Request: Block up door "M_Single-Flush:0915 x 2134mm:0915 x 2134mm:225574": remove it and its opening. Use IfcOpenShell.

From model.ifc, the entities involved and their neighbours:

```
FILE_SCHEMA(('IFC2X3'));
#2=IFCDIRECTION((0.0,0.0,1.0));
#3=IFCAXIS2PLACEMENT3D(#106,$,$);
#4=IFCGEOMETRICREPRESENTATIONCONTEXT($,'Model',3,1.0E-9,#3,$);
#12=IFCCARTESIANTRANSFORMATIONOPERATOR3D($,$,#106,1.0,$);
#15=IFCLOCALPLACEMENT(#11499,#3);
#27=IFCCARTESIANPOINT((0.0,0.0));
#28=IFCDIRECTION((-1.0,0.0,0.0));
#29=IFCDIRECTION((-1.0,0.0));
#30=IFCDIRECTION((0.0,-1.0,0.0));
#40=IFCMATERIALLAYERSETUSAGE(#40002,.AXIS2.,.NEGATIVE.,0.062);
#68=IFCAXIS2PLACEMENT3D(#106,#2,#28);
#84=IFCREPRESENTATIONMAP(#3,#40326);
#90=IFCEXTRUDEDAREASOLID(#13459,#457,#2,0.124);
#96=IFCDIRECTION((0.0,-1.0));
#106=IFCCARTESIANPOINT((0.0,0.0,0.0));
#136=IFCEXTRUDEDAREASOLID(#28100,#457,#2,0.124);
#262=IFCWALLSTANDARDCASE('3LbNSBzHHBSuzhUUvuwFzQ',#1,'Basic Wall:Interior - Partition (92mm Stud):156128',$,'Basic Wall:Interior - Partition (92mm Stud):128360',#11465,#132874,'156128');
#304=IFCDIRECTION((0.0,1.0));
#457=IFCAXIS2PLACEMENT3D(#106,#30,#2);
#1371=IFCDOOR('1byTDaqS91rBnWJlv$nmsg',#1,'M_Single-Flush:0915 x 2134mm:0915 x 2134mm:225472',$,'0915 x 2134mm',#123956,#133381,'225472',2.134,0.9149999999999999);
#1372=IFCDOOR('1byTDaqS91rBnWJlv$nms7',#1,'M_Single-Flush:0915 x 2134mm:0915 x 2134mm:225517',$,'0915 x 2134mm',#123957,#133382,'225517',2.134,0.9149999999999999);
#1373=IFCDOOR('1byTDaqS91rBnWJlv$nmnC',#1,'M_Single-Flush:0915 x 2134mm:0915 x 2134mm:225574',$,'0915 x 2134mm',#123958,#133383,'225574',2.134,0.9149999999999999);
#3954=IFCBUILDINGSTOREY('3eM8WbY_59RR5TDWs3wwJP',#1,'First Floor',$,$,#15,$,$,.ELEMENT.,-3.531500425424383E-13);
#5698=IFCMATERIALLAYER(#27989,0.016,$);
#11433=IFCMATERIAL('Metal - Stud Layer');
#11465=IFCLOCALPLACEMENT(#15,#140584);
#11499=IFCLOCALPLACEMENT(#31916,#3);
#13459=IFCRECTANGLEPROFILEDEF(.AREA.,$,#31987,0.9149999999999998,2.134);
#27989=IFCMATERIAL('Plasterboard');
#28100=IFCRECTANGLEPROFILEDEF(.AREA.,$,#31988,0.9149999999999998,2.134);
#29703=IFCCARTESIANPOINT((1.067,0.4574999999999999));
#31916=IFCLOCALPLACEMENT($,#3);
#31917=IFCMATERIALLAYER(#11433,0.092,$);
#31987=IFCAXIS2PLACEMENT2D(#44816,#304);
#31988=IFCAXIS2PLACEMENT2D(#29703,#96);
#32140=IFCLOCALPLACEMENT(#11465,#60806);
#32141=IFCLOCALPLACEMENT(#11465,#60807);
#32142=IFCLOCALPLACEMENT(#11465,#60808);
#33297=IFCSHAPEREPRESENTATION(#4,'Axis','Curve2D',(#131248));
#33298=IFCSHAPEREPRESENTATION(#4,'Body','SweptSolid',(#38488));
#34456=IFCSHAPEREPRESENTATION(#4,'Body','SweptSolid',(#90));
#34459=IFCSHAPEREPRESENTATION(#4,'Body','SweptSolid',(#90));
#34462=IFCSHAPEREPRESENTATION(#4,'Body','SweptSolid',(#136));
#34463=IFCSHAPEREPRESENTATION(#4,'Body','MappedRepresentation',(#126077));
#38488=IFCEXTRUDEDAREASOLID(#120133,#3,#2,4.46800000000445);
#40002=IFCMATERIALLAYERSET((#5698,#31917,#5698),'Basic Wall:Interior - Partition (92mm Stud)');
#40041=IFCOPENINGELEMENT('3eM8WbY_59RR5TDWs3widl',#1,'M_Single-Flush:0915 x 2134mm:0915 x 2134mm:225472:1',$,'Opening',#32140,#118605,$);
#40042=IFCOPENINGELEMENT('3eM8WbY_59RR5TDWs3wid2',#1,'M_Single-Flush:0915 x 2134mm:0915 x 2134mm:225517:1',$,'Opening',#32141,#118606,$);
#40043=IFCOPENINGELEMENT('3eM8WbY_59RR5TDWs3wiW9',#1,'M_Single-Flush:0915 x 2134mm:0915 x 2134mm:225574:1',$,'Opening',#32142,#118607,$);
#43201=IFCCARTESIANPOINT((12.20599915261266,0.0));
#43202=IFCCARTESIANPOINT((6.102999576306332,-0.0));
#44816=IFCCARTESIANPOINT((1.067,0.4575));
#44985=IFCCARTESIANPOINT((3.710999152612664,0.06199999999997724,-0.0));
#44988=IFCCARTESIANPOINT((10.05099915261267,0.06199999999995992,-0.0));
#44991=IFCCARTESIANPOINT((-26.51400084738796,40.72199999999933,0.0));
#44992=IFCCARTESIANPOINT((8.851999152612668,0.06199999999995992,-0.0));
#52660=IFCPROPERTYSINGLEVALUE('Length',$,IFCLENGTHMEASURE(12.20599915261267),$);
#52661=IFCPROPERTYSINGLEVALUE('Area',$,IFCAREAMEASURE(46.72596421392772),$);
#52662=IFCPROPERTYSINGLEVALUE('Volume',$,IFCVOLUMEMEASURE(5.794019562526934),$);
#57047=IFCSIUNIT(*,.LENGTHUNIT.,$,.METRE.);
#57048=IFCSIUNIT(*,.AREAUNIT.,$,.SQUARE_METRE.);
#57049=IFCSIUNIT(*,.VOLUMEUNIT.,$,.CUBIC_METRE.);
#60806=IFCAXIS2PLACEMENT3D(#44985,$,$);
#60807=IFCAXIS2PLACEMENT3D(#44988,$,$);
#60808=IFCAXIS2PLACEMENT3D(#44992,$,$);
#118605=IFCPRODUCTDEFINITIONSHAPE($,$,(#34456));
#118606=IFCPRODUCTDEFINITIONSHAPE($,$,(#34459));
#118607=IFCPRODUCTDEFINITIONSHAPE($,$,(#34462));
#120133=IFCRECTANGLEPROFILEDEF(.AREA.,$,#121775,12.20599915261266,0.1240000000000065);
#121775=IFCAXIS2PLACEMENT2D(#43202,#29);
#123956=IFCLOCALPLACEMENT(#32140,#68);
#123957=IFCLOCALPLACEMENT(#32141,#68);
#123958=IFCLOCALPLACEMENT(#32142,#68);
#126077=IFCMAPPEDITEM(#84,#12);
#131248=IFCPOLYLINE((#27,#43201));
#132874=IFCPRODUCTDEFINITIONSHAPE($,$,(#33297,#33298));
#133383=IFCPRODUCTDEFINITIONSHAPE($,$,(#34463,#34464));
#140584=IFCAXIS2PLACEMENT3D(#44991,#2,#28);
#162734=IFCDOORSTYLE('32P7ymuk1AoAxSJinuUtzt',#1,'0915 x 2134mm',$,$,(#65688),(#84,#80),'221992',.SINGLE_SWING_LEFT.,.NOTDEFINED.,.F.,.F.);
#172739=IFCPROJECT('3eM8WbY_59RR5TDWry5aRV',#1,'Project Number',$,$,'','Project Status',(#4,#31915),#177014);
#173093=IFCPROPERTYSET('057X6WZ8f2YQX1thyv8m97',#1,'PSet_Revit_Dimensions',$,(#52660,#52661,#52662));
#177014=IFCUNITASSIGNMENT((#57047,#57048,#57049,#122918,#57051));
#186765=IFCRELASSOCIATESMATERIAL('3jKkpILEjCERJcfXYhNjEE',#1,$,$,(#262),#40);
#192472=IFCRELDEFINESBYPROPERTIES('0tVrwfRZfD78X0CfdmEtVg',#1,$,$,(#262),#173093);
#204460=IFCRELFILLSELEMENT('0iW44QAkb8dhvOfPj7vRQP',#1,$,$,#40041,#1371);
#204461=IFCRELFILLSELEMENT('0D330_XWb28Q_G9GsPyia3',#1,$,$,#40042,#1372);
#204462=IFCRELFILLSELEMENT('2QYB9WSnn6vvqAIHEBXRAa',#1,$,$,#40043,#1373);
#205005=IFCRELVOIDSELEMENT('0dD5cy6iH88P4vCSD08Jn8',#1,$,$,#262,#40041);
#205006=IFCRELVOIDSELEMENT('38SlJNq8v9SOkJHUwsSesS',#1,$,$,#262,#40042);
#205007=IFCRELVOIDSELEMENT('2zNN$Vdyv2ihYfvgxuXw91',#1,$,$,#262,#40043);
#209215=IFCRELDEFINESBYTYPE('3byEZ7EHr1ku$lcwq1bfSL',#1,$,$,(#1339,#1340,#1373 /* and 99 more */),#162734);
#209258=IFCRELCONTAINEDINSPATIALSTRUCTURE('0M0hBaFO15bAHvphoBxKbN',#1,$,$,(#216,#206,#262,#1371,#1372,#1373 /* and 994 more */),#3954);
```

```python
import ifcopenshell
import ifcopenshell.api.feature
import ifcopenshell.api.pset
import ifcopenshell.api.root
import ifcopenshell.geom
import ifcopenshell.util.element
import ifcopenshell.util.shape
import ifcopenshell.util.unit

model = ifcopenshell.open("model.ifc")
area_scale = ifcopenshell.util.unit.calculate_unit_scale(model, "AREAUNIT")
volume_scale = ifcopenshell.util.unit.calculate_unit_scale(model, "VOLUMEUNIT")
settings = ifcopenshell.geom.settings()


def volume(element):
    """Net volume in cubic metres, openings subtracted."""
    shape = ifcopenshell.geom.create_shape(settings, element)
    return ifcopenshell.util.shape.get_volume(shape.geometry)


door = model.by_guid("1byTDaqS91rBnWJlv$nmnC")
opening = door.FillsVoids[0].RelatingOpeningElement
wall = opening.VoidsElements[0].RelatingBuildingElement
before = volume(wall)

ifcopenshell.api.root.remove_product(model, product=door)
ifcopenshell.api.feature.remove_feature(model, feature=opening)

after = volume(wall)
thickness = 0.124  # wall thickness in metres

# Update the wall's stored quantities.
pset = model.by_id(ifcopenshell.util.element.get_pset(wall, "PSet_Revit_Dimensions", should_inherit=False)["id"])
ifcopenshell.api.pset.edit_pset(model, pset=pset, properties={
    "Area": model.create_entity("IfcAreaMeasure", after / thickness / area_scale),
    "Volume": model.create_entity("IfcVolumeMeasure", after / volume_scale),
})

print(f"wall volume {before:.3f} -> {after:.3f} m3")

model.write("model_rev.ifc")
```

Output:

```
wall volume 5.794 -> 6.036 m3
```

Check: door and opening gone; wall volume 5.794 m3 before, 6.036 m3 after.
